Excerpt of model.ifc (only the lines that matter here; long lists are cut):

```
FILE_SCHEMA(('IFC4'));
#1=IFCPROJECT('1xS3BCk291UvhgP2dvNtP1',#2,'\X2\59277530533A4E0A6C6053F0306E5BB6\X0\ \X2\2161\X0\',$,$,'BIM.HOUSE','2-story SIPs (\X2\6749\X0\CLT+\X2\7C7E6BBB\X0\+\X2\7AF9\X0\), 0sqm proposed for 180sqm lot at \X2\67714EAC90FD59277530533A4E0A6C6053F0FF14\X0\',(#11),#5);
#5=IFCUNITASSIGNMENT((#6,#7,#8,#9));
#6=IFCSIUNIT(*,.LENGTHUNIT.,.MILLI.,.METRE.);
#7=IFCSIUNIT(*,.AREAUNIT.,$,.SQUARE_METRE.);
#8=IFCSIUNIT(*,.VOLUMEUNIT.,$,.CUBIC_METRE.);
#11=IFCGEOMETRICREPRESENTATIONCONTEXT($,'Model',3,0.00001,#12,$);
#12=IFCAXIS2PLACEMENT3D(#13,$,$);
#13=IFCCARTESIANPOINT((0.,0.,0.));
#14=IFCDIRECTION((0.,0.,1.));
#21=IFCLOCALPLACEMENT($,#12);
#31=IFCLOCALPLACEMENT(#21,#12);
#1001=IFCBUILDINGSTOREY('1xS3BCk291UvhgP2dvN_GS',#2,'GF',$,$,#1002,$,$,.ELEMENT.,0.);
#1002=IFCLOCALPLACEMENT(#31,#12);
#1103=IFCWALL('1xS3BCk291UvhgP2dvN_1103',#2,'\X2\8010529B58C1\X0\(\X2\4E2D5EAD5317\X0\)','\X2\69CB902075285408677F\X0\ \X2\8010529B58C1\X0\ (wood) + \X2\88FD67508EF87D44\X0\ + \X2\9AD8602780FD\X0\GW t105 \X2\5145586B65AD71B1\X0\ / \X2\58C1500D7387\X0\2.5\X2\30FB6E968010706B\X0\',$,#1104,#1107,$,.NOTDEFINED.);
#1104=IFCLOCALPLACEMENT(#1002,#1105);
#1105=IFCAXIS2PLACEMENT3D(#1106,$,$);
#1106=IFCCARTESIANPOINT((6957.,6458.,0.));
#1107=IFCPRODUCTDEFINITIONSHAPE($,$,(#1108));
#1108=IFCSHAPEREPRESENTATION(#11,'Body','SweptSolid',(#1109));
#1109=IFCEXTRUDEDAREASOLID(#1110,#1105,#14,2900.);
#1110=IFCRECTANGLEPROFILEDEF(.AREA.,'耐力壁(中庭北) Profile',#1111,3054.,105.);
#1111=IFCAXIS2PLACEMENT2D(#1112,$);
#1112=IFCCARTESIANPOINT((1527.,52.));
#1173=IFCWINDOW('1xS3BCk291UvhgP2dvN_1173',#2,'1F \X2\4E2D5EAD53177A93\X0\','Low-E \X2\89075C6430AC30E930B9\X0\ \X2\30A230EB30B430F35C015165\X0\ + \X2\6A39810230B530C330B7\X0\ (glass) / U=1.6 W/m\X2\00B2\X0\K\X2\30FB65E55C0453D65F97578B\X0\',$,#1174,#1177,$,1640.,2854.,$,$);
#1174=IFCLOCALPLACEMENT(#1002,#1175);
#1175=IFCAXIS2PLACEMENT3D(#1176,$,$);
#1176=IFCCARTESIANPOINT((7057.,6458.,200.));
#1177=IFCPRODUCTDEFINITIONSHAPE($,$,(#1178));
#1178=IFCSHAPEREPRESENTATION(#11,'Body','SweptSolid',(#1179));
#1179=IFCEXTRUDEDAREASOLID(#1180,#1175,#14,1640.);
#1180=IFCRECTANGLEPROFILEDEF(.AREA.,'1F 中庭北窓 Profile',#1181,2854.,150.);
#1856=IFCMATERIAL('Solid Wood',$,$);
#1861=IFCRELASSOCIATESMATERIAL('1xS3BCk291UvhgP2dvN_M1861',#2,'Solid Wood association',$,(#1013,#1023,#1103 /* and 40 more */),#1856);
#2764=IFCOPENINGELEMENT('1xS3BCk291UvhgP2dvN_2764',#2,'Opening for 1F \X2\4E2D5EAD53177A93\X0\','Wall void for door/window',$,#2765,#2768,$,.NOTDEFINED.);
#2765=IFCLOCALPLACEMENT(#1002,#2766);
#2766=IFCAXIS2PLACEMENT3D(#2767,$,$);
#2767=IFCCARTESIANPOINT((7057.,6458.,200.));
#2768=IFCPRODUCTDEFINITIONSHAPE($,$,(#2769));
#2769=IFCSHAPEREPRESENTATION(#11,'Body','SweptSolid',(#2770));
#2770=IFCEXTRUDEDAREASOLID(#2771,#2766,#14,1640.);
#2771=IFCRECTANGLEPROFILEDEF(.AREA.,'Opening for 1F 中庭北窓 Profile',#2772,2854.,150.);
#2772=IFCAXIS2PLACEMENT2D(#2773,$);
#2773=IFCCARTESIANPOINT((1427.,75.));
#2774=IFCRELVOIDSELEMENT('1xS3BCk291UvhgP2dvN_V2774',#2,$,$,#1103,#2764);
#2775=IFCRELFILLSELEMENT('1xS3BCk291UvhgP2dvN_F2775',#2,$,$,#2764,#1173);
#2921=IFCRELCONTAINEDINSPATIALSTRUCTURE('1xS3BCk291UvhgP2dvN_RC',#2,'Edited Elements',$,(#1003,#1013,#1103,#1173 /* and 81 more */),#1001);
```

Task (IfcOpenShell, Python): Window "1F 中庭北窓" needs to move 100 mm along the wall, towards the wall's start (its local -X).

```python
import ifcopenshell
import ifcopenshell.api.geometry
import ifcopenshell.util.placement
import ifcopenshell.util.unit

model = ifcopenshell.open("model.ifc")
unit_scale = ifcopenshell.util.unit.calculate_unit_scale(model)

window = model.by_guid("1xS3BCk291UvhgP2dvN_1173")
opening = window.FillsVoids[0].RelatingOpeningElement
wall = opening.VoidsElements[0].RelatingBuildingElement

wall_matrix = ifcopenshell.util.placement.get_local_placement(wall.ObjectPlacement)
shift = wall_matrix[:3, 0] * -0.1 / unit_scale
before = ifcopenshell.util.placement.get_local_placement(window.ObjectPlacement)[:3, 3].copy()

# The window is not placed relative to its opening, so move both.
for product in (opening, window):
    matrix = ifcopenshell.util.placement.get_local_placement(product.ObjectPlacement)
    matrix[:3, 3] += shift
    ifcopenshell.api.geometry.edit_object_placement(model, product=product, matrix=matrix, is_si=False)

after = ifcopenshell.util.placement.get_local_placement(window.ObjectPlacement)[:3, 3]
print("window moved by", (after - before).round(3) + 0.0)

model.write("model-out.ifc")
```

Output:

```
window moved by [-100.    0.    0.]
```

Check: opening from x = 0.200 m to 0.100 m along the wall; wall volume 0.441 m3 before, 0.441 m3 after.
